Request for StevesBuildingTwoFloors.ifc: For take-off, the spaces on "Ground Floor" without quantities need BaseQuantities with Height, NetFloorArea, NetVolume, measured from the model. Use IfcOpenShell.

First a look at what the model holds.

```python
import ifcopenshell
import ifcopenshell.util.element
import ifcopenshell.util.unit

model = ifcopenshell.open("StevesBuildingTwoFloors.ifc")
print(model.schema)
for unit_type in ("LENGTHUNIT", "AREAUNIT", "VOLUMEUNIT"):
    print(unit_type, ifcopenshell.util.unit.calculate_unit_scale(model, unit_type))
storey = next(s for s in model.by_type("IfcBuildingStorey") if s.Name == "Ground Floor")
spaces = [e for e in ifcopenshell.util.element.get_decomposition(storey) if e.is_a("IfcSpace")]
for e in sorted(spaces, key=lambda e: e.id()):
    print(e.id(), e.is_a(), e.Name, list(ifcopenshell.util.element.get_psets(e, qtos_only=True)), sep=" | ")
```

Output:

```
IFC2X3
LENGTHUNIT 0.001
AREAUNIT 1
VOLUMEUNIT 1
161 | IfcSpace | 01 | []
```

```python
import ifcopenshell
import ifcopenshell.api.pset
import ifcopenshell.geom
import ifcopenshell.util.element
import ifcopenshell.util.shape
import ifcopenshell.util.unit

model = ifcopenshell.open("StevesBuildingTwoFloors.ifc")
unit_scale = ifcopenshell.util.unit.calculate_unit_scale(model)
area_scale = ifcopenshell.util.unit.calculate_unit_scale(model, "AREAUNIT")
volume_scale = ifcopenshell.util.unit.calculate_unit_scale(model, "VOLUMEUNIT")
settings = ifcopenshell.geom.settings()

storey = next(s for s in model.by_type("IfcBuildingStorey") if s.Name == "Ground Floor")
spaces = [e for e in ifcopenshell.util.element.get_decomposition(storey) if e.is_a("IfcSpace")]

for e in sorted(spaces, key=lambda e: e.id()):
    if ifcopenshell.util.element.get_psets(e, qtos_only=True, should_inherit=False):
        continue
    # Geometry comes back in metres, in the element's own axes.
    shape = ifcopenshell.geom.create_shape(settings, e)
    values = {
        "Height": ifcopenshell.util.shape.get_z(shape.geometry) / unit_scale,
        "NetFloorArea": ifcopenshell.util.shape.get_footprint_area(shape.geometry) / area_scale,
        "NetVolume": ifcopenshell.util.shape.get_volume(shape.geometry) / volume_scale,
    }
    qto = ifcopenshell.api.pset.add_qto(model, product=e, name="BaseQuantities")
    ifcopenshell.api.pset.edit_qto(model, qto=qto, properties=values)
    print(e.id(), {k: round(v, 3) for k, v in values.items()})

model.write("StevesBuildingTwoFloors_rev.ifc")
```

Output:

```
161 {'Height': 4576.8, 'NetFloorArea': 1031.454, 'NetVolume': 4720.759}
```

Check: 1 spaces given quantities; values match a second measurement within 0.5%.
